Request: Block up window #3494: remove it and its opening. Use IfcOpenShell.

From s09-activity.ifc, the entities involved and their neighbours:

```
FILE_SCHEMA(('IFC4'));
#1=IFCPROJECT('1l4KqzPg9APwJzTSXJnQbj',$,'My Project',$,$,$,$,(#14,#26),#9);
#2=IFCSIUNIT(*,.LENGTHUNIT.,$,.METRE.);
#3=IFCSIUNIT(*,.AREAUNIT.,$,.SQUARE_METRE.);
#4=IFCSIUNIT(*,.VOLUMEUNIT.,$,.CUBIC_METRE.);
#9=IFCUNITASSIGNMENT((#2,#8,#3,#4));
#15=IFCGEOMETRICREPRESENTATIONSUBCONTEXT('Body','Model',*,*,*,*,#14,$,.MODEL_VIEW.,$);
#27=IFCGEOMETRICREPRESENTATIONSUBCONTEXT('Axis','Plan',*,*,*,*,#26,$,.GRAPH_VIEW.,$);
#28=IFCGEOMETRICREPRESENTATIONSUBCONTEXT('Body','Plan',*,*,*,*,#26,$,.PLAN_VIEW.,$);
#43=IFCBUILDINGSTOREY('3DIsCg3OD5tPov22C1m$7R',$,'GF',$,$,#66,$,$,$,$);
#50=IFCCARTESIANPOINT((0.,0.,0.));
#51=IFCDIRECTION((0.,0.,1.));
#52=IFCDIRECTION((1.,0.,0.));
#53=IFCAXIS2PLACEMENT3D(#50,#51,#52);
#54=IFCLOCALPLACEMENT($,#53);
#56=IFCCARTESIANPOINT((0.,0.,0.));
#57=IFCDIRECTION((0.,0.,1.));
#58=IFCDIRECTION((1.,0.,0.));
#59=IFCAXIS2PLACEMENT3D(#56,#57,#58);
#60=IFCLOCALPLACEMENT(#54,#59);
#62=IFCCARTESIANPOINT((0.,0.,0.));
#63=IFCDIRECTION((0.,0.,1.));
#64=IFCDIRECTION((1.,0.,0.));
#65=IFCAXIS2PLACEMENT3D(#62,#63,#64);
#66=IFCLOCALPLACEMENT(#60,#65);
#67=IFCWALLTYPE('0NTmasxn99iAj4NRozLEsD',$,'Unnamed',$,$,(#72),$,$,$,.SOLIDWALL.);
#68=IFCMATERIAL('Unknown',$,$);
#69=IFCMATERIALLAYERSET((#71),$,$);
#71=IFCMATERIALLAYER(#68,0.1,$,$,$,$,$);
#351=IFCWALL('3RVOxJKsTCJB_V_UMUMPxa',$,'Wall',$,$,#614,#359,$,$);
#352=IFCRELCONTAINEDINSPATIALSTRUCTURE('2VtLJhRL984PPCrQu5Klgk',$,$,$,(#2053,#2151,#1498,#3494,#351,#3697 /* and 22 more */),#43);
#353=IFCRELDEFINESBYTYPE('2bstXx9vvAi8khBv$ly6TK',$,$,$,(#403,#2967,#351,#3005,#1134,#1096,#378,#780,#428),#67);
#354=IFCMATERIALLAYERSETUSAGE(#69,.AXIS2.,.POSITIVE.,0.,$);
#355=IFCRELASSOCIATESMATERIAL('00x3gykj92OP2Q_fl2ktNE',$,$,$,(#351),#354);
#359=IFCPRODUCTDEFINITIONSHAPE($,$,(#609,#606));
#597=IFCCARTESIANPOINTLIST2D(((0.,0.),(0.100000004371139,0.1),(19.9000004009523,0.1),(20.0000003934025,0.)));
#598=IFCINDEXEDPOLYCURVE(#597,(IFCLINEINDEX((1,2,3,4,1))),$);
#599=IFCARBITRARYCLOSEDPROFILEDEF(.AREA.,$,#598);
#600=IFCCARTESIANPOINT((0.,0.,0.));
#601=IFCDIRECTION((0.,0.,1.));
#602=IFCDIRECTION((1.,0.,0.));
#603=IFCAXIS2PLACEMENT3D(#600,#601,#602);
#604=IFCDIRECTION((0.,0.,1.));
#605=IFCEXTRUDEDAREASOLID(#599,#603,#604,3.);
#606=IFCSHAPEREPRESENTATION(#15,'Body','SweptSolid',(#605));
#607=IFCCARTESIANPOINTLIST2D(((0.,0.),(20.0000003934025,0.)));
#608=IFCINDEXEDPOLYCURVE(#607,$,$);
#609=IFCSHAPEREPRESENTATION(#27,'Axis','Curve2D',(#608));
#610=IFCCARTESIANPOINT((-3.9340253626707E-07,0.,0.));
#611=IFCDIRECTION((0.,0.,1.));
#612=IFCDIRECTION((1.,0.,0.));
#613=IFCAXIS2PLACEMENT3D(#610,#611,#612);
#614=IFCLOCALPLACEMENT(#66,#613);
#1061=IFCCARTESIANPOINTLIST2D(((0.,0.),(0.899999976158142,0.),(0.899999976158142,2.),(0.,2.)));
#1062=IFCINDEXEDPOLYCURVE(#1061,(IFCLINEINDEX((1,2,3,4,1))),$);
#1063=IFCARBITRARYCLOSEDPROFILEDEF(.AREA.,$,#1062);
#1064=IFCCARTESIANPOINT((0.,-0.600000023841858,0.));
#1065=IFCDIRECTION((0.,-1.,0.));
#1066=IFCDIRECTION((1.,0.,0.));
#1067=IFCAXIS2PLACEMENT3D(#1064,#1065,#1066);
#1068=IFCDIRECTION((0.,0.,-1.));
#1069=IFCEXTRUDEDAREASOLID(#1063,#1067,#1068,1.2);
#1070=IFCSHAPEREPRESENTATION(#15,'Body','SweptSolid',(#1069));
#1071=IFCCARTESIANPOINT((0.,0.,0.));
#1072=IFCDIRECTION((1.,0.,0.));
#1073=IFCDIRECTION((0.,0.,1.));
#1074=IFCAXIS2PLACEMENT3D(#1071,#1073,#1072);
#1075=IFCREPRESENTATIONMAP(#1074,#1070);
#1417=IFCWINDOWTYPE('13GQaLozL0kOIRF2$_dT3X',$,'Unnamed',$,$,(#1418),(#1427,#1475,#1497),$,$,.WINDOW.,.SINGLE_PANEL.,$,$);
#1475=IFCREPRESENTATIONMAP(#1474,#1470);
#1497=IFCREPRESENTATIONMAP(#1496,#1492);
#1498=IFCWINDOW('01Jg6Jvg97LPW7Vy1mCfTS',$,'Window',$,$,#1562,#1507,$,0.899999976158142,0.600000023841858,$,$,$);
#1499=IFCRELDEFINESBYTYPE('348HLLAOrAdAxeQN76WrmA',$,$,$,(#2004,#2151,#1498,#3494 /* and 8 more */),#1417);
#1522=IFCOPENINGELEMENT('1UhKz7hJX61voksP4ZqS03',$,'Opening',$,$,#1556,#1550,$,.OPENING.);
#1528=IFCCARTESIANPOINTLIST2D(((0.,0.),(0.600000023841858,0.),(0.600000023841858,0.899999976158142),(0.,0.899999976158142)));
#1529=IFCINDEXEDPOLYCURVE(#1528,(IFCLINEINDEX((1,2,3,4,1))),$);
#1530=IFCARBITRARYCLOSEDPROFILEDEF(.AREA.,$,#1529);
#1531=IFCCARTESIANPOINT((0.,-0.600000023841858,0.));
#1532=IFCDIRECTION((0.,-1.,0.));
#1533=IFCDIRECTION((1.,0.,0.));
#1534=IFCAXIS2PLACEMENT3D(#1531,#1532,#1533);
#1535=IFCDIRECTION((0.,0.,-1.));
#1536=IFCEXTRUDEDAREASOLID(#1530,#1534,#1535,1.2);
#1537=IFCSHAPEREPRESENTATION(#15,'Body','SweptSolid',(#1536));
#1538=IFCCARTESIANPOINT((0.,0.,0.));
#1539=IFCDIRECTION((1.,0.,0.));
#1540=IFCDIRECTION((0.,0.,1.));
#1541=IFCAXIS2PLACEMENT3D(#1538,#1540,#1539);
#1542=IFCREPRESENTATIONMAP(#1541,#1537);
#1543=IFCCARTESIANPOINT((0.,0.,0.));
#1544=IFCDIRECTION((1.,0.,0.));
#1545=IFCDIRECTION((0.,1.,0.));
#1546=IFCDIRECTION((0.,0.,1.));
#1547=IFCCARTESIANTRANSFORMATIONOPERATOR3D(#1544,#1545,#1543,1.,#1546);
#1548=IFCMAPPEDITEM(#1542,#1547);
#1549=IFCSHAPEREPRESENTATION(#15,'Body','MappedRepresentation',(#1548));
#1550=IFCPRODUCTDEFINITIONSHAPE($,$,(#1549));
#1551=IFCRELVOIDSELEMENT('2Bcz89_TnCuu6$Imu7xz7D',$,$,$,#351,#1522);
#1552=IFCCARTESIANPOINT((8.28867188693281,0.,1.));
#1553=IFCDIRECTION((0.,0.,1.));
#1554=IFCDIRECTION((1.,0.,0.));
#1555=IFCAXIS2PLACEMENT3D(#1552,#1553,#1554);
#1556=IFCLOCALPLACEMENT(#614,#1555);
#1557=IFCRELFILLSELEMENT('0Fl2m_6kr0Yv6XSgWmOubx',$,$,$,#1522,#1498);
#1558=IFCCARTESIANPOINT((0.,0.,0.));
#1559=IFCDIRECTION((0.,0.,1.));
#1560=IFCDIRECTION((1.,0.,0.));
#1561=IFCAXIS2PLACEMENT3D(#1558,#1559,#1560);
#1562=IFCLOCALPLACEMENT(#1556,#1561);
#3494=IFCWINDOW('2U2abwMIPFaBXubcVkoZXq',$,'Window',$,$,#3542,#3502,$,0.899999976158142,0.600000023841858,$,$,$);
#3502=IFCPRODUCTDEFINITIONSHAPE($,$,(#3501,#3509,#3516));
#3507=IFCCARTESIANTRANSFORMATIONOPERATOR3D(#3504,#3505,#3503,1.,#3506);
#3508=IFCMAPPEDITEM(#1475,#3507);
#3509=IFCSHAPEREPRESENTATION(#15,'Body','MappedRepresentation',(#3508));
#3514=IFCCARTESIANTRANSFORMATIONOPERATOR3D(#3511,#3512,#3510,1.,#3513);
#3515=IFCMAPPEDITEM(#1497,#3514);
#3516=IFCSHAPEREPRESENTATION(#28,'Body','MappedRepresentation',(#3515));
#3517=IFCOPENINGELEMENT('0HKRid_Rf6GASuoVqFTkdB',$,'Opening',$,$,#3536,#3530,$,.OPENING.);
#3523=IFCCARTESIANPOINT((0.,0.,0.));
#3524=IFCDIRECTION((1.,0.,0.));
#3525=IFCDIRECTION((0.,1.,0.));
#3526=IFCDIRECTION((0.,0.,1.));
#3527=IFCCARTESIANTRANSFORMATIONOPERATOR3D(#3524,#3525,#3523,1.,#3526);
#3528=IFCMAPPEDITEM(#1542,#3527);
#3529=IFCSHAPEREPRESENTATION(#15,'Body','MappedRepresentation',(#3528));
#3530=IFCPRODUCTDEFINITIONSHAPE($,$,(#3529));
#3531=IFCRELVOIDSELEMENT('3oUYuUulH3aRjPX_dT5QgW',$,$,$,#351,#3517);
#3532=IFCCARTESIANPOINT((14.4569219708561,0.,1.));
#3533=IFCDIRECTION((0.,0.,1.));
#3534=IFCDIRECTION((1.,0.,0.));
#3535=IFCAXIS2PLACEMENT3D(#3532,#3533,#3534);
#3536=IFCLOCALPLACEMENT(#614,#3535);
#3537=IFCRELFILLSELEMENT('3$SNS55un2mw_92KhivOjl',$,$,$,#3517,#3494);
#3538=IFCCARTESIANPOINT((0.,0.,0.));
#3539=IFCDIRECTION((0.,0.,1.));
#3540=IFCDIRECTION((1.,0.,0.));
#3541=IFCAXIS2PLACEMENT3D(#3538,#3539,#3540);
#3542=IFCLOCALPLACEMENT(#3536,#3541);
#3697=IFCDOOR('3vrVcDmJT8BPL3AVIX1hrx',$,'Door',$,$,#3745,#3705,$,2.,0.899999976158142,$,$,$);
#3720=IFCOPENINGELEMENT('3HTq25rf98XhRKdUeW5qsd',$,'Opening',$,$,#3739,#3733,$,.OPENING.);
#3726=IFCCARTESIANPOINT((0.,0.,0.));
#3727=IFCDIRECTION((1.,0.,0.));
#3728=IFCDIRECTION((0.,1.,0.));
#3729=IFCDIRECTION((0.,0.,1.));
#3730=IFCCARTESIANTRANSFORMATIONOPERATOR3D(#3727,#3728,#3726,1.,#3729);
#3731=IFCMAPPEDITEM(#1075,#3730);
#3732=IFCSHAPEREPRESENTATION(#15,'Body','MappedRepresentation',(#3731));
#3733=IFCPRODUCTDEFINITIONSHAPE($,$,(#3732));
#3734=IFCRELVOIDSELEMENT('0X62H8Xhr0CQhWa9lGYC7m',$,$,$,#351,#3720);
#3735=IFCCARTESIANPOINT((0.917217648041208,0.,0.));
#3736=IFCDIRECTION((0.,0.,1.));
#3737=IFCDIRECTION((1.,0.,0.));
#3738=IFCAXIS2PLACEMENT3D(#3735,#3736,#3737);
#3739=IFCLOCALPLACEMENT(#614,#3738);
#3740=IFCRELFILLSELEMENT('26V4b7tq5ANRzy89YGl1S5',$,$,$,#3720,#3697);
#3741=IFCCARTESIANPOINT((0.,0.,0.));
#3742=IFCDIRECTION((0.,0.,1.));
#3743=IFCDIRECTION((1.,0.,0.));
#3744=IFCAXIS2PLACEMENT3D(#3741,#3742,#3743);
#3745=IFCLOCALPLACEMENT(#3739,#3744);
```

```python
import ifcopenshell
import ifcopenshell.api.feature
import ifcopenshell.api.root
import ifcopenshell.geom
import ifcopenshell.util.shape

model = ifcopenshell.open("s09-activity.ifc")
settings = ifcopenshell.geom.settings()


def volume(element):
    """Net volume in cubic metres, openings subtracted."""
    shape = ifcopenshell.geom.create_shape(settings, element)
    return ifcopenshell.util.shape.get_volume(shape.geometry)


window = model.by_guid("2U2abwMIPFaBXubcVkoZXq")
opening = window.FillsVoids[0].RelatingOpeningElement
wall = opening.VoidsElements[0].RelatingBuildingElement
before = volume(wall)

ifcopenshell.api.root.remove_product(model, product=window)
ifcopenshell.api.feature.remove_feature(model, feature=opening)

after = volume(wall)

print(f"wall volume {before:.3f} -> {after:.3f} m3")

model.write("s09-activity_updated.ifc")
```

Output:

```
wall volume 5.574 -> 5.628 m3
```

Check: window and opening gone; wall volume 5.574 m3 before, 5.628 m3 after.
